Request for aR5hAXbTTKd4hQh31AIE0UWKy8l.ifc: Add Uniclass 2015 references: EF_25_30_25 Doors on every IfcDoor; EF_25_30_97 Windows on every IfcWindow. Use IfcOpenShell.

First a look at what the model holds.

```python
import ifcopenshell

model = ifcopenshell.open("aR5hAXbTTKd4hQh31AIE0UWKy8l.ifc")
print(model.schema)
print("classifications:", [c.Name for c in model.by_type("IfcClassification")])
for ifc_class in ("IfcDoor", "IfcRoof", "IfcStair", "IfcWall", "IfcWindow"):
    print(ifc_class, len(model.by_type(ifc_class)))
```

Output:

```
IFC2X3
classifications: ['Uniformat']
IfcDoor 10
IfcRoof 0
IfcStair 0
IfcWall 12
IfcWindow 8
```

```python
import ifcopenshell
import ifcopenshell.api.classification

model = ifcopenshell.open("aR5hAXbTTKd4hQh31AIE0UWKy8l.ifc")

# IFC2X3 requires Source and Edition and has no link from the project to the system.
system = model.create_entity("IfcClassification", Source="NBS", Edition="2015", Name="Uniclass 2015")

codes = {
    "IfcDoor": ("EF_25_30_25", "Doors"),
    "IfcWindow": ("EF_25_30_97", "Windows"),
}
for ifc_class, (code, name) in codes.items():
    products = model.by_type(ifc_class)
    ifcopenshell.api.classification.add_reference(
        model, products=products, classification=system, identification=code, name=name
    )
    print(code, len(products))

model.write("aR5hAXbTTKd4hQh31AIE0UWKy8l-out.ifc")
```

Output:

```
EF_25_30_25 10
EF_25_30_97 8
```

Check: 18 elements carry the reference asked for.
